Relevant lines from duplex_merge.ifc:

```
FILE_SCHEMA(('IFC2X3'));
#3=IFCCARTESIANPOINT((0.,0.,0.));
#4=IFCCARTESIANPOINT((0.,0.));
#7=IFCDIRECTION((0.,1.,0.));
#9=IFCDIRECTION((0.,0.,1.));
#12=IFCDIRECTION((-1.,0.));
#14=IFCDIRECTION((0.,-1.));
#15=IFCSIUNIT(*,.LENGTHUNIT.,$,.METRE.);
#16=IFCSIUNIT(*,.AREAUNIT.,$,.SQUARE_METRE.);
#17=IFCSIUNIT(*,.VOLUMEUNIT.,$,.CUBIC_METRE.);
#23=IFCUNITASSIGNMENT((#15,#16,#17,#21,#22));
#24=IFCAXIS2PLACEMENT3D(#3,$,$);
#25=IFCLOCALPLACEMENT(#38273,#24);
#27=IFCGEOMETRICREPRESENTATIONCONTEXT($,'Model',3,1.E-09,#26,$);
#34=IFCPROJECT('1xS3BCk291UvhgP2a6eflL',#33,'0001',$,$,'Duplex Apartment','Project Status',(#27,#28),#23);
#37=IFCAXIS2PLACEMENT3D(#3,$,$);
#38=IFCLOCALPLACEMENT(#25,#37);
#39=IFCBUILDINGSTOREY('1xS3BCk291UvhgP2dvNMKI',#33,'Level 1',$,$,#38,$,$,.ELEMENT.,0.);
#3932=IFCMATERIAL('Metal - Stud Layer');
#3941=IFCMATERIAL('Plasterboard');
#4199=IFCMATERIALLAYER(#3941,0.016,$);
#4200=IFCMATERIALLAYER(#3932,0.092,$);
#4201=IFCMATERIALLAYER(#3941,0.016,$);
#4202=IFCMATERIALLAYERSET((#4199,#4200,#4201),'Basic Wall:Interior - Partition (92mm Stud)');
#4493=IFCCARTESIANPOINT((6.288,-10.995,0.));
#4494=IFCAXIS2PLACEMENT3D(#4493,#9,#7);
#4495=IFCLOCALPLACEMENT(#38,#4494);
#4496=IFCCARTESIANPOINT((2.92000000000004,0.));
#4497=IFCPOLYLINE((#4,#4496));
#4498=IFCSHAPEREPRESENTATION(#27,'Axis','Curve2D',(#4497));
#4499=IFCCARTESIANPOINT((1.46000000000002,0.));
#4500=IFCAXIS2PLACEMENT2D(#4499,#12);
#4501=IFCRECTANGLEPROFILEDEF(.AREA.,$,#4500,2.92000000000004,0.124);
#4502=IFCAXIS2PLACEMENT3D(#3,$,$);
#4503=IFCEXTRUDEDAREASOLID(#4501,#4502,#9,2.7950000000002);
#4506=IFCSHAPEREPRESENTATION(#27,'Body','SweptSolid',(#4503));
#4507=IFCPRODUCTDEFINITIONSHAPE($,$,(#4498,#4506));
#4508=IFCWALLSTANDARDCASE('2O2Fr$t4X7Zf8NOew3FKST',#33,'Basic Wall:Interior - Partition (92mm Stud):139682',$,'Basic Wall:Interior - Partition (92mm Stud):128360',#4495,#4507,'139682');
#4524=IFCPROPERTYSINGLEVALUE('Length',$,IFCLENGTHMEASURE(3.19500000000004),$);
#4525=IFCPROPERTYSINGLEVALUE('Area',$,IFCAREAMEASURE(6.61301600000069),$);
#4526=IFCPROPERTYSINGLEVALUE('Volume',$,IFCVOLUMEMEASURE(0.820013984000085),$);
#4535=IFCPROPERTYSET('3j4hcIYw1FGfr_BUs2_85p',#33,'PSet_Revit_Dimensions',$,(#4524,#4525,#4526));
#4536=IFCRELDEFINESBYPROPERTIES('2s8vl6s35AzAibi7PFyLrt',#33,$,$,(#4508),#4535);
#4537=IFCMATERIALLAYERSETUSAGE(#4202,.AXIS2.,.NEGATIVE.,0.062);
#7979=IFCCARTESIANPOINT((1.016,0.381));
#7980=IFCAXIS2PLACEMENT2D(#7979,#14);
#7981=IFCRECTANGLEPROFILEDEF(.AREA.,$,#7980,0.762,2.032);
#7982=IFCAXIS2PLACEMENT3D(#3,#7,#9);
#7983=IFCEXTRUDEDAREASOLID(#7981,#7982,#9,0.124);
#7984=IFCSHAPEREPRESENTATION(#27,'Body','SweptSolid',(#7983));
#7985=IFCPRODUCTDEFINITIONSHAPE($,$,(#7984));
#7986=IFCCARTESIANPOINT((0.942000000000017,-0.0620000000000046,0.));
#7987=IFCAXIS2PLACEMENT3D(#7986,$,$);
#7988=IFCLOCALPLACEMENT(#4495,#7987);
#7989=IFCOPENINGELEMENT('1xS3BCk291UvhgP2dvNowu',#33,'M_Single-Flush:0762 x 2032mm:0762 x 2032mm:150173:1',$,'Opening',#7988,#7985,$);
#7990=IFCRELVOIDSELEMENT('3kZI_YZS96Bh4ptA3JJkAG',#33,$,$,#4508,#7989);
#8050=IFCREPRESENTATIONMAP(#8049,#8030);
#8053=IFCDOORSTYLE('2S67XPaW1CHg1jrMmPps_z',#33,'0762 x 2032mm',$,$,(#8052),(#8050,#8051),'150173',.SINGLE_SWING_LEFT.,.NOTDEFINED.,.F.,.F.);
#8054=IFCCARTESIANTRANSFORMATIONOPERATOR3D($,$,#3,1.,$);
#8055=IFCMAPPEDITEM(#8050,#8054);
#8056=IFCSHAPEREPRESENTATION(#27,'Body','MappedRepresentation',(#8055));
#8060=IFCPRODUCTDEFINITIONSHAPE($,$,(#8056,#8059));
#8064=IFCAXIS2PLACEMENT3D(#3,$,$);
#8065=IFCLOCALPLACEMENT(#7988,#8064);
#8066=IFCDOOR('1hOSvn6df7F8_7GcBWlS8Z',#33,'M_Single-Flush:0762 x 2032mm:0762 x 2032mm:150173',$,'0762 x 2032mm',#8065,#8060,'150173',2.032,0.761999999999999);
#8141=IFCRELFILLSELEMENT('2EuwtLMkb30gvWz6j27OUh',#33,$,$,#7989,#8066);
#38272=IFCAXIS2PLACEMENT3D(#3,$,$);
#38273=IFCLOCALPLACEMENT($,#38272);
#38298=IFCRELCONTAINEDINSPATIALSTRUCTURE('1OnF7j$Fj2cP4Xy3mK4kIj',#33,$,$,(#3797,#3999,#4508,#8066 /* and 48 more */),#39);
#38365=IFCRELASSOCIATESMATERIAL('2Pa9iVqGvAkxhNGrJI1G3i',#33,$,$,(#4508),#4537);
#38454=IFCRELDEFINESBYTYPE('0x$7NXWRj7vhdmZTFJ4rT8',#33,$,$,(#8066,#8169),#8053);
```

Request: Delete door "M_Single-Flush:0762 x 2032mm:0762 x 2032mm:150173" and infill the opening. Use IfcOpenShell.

```python
import ifcopenshell
import ifcopenshell.api.feature
import ifcopenshell.api.pset
import ifcopenshell.api.root
import ifcopenshell.geom
import ifcopenshell.util.element
import ifcopenshell.util.shape
import ifcopenshell.util.unit

model = ifcopenshell.open("duplex_merge.ifc")
area_scale = ifcopenshell.util.unit.calculate_unit_scale(model, "AREAUNIT")
volume_scale = ifcopenshell.util.unit.calculate_unit_scale(model, "VOLUMEUNIT")
settings = ifcopenshell.geom.settings()


def volume(element):
    """Net volume in cubic metres, openings subtracted."""
    shape = ifcopenshell.geom.create_shape(settings, element)
    return ifcopenshell.util.shape.get_volume(shape.geometry)


door = model.by_guid("1hOSvn6df7F8_7GcBWlS8Z")
opening = door.FillsVoids[0].RelatingOpeningElement
wall = opening.VoidsElements[0].RelatingBuildingElement
before = volume(wall)

ifcopenshell.api.root.remove_product(model, product=door)
ifcopenshell.api.feature.remove_feature(model, feature=opening)

after = volume(wall)
thickness = 0.124  # wall thickness in metres

# Update the wall's stored quantities.
pset = model.by_id(ifcopenshell.util.element.get_pset(wall, "PSet_Revit_Dimensions", should_inherit=False)["id"])
ifcopenshell.api.pset.edit_pset(model, pset=pset, properties={
    "Area": model.create_entity("IfcAreaMeasure", after / thickness / area_scale),
    "Volume": model.create_entity("IfcVolumeMeasure", after / volume_scale),
})

print(f"wall volume {before:.3f} -> {after:.3f} m3")

model.write("duplex_merge_rev.ifc")
```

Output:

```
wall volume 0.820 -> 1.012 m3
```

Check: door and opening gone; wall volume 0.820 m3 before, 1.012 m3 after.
